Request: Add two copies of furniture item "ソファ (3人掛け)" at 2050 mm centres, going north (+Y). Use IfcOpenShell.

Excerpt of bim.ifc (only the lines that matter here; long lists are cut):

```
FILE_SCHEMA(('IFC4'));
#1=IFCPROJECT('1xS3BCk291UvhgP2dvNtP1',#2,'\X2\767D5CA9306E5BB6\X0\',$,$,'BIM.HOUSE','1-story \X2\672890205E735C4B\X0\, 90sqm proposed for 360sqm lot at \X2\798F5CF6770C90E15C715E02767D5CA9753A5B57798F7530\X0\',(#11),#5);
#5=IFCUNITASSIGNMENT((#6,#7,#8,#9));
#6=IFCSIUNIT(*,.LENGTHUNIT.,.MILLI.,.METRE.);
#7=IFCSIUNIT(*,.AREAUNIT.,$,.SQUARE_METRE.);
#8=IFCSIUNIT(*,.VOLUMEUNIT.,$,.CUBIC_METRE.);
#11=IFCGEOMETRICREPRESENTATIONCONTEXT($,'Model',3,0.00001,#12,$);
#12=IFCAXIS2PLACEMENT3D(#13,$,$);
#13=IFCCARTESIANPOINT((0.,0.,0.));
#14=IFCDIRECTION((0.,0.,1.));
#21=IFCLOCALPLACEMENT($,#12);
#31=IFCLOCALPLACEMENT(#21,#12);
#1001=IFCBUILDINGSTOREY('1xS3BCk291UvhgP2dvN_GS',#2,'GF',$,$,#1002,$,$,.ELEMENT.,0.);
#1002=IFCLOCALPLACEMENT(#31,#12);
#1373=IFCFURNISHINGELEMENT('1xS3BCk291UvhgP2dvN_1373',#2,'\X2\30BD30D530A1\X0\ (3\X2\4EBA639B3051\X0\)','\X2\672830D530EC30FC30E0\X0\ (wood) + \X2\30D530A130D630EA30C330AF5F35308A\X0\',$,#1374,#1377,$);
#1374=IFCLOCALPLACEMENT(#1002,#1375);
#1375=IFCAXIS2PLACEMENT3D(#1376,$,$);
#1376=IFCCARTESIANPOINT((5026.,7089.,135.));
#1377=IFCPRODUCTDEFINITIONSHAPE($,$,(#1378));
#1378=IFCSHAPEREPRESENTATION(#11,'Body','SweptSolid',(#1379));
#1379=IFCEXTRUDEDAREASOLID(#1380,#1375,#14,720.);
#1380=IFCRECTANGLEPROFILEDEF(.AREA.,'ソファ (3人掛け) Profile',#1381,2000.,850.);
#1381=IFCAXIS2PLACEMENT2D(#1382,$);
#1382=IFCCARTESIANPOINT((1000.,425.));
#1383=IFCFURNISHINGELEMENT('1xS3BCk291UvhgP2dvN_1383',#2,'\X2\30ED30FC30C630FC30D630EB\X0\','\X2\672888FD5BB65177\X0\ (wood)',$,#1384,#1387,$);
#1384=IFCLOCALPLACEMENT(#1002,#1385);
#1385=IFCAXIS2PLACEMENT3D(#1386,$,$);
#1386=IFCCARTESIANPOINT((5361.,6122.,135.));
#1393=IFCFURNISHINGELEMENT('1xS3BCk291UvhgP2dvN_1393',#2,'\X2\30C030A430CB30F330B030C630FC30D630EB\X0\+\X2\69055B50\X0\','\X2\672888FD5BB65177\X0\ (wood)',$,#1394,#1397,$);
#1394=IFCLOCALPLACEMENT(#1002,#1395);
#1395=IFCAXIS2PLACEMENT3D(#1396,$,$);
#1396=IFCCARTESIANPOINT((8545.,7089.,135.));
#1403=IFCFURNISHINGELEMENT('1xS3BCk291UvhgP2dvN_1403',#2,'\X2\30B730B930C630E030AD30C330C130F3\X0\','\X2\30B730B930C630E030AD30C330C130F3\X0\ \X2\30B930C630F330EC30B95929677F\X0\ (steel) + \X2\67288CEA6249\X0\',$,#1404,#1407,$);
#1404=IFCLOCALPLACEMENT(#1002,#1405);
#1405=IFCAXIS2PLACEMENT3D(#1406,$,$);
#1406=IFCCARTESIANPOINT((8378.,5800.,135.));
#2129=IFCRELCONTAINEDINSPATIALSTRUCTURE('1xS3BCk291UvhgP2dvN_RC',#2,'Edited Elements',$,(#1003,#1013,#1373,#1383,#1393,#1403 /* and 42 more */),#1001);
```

```python
import numpy as np
import ifcopenshell
import ifcopenshell.api.geometry
import ifcopenshell.api.root
import ifcopenshell.util.element
import ifcopenshell.util.placement

model = ifcopenshell.open("bim.ifc")


def reuse_history(source, copy):
    """copy_class also copies each property set's owner history, people and application; keep the originals."""
    for rel in copy.IsDefinedBy:
        if rel.is_a("IfcRelDefinesByProperties") and (history := rel.RelatingPropertyDefinition.OwnerHistory):
            rel.RelatingPropertyDefinition.OwnerHistory = source.OwnerHistory
            ifcopenshell.util.element.remove_deep2(model, history)


source = model.by_guid("1xS3BCk291UvhgP2dvN_1373")
base = ifcopenshell.util.placement.get_local_placement(source.ObjectPlacement)
step = np.array([0.0, 1.0, 0.0]) * 2050.0

for i in range(1, 3):
    copy = ifcopenshell.api.root.copy_class(model, product=source)
    copy.Representation = ifcopenshell.util.element.copy_deep(
        model, source.Representation, exclude=["IfcGeometricRepresentationContext", "IfcRepresentationMap"]
    )
    reuse_history(source, copy)
    matrix = base.copy()
    matrix[:3, 3] += i * step
    print("added at", matrix[:3, 3].round(3) + 0.0)
    ifcopenshell.api.geometry.edit_object_placement(model, product=copy, matrix=matrix, is_si=False)

model.write("bim_rev.ifc")
```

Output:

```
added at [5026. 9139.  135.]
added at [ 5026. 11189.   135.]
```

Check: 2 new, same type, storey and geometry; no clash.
